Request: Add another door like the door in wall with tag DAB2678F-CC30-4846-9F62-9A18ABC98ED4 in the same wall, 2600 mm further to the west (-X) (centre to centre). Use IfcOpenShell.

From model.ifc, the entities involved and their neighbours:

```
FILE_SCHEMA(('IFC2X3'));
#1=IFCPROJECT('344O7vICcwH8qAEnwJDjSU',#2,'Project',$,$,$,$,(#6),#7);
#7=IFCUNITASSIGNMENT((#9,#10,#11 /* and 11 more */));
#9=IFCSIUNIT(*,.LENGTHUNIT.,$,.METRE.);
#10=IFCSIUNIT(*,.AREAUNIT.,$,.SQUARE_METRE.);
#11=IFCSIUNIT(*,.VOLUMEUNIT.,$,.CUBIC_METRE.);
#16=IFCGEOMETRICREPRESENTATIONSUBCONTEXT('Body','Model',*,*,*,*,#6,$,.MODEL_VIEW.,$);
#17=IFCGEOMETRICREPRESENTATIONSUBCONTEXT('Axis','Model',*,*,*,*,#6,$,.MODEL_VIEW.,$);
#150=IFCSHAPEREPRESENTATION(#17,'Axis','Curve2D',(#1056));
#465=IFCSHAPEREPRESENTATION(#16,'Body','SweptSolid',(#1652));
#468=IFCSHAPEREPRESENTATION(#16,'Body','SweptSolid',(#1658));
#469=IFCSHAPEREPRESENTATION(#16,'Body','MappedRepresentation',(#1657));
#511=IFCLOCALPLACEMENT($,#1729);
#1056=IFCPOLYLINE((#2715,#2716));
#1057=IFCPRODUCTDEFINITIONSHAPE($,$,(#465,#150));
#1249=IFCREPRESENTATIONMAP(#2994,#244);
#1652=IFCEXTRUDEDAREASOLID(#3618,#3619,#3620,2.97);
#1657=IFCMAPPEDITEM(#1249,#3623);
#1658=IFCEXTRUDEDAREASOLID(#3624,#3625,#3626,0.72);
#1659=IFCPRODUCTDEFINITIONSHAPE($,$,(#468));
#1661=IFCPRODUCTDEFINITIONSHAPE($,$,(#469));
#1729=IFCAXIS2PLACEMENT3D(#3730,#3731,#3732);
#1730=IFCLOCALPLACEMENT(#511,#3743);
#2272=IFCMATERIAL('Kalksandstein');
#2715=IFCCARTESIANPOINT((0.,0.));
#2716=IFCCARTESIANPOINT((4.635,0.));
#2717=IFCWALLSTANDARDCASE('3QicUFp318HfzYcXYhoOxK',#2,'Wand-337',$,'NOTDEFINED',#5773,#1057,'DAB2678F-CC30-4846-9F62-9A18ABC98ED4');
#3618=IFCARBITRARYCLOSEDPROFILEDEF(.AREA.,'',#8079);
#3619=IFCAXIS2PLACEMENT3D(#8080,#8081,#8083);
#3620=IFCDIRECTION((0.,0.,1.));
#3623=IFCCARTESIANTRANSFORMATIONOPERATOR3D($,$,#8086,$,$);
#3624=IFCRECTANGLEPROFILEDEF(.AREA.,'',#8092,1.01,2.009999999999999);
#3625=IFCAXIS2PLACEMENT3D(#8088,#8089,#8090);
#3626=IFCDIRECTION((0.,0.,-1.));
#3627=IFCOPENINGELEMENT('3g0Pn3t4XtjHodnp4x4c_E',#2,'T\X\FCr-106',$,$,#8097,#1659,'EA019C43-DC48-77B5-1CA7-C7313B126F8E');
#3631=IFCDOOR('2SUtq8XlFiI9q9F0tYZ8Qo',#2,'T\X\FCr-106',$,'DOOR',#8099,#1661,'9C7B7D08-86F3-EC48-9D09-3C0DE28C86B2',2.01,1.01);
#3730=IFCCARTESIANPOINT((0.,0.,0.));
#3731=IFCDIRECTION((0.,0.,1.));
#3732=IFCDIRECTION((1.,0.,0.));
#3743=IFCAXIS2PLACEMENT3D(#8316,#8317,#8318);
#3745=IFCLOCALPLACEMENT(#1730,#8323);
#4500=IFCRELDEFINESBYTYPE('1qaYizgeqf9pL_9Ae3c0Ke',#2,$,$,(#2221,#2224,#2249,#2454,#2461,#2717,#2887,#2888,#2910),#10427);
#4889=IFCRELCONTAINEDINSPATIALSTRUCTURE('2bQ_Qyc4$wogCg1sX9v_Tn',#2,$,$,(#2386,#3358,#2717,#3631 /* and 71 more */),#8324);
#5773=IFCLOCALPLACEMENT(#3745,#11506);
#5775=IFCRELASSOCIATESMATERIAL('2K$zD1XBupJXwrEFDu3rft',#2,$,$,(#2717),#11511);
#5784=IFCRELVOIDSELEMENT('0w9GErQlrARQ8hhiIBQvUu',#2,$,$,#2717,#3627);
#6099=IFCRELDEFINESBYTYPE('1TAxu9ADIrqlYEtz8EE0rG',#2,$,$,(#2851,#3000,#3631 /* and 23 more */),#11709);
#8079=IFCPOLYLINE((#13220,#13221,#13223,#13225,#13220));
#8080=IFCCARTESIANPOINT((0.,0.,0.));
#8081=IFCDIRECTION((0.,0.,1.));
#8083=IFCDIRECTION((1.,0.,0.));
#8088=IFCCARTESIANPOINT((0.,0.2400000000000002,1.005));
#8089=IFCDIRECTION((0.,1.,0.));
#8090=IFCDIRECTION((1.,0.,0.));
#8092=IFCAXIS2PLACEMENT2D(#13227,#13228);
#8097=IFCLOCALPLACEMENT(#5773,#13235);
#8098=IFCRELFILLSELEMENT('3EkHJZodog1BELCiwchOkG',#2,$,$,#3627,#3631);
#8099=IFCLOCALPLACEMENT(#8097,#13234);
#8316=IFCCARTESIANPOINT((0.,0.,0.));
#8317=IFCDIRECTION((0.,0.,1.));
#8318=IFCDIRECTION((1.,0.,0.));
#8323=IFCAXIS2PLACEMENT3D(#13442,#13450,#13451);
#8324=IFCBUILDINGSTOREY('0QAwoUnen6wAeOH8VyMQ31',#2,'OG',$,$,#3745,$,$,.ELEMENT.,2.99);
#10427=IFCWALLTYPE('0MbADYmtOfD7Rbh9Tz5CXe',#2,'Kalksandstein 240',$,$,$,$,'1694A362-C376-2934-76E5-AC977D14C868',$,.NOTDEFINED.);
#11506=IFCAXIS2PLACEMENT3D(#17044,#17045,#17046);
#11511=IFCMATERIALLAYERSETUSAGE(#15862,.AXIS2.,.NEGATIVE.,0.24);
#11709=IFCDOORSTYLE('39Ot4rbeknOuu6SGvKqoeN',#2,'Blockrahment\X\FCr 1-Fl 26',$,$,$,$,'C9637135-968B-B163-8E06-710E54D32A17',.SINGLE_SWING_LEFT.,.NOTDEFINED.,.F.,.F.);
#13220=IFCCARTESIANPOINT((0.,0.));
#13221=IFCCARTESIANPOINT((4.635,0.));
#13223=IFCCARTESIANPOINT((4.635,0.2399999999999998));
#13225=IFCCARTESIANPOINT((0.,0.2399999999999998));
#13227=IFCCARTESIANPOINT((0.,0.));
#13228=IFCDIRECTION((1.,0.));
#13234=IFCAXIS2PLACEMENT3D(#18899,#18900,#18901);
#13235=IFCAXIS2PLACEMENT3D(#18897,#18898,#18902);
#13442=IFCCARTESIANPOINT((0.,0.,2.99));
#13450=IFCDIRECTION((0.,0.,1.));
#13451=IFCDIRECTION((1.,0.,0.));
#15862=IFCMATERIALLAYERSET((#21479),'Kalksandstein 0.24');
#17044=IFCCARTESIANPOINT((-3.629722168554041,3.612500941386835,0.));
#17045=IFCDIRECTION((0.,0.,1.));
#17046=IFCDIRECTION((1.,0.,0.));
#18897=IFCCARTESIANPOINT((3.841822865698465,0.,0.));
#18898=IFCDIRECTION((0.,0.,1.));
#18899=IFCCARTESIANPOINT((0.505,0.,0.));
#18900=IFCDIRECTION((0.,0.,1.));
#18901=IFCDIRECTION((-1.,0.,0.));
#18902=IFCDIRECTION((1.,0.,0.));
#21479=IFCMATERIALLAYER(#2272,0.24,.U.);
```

```python
import ifcopenshell
import ifcopenshell.api.feature
import ifcopenshell.api.geometry
import ifcopenshell.api.root
import ifcopenshell.geom
import ifcopenshell.util.element
import ifcopenshell.util.placement
import ifcopenshell.util.shape
import ifcopenshell.util.unit

model = ifcopenshell.open("model.ifc")
unit_scale = ifcopenshell.util.unit.calculate_unit_scale(model)
settings = ifcopenshell.geom.settings()


def volume(element):
    """Net volume in cubic metres, openings subtracted."""
    shape = ifcopenshell.geom.create_shape(settings, element)
    return ifcopenshell.util.shape.get_volume(shape.geometry)


def reuse_history(source, copy):
    """copy_class also copies each property set's owner history, people and application; keep the originals."""
    for rel in copy.IsDefinedBy:
        if rel.is_a("IfcRelDefinesByProperties") and (history := rel.RelatingPropertyDefinition.OwnerHistory):
            rel.RelatingPropertyDefinition.OwnerHistory = source.OwnerHistory
            ifcopenshell.util.element.remove_deep2(model, history)


door = model.by_guid("2SUtq8XlFiI9q9F0tYZ8Qo")
opening = door.FillsVoids[0].RelatingOpeningElement
wall = opening.VoidsElements[0].RelatingBuildingElement
before = volume(wall)
shift = ifcopenshell.util.placement.get_local_placement(wall.ObjectPlacement)[:3, 0] * -2.6 / unit_scale

# copy_class copies the void relationship, type, container and properties, but no geometry.
new_opening = ifcopenshell.api.root.copy_class(model, product=opening)
new_opening.Representation = ifcopenshell.util.element.copy_deep(
    model, opening.Representation, exclude=["IfcGeometricRepresentationContext", "IfcRepresentationMap"]
)
new_opening.Tag = None
new_door = ifcopenshell.api.root.copy_class(model, product=door)
new_door.Representation = ifcopenshell.util.element.copy_deep(
    model, door.Representation, exclude=["IfcGeometricRepresentationContext", "IfcRepresentationMap"]
)
new_door.Tag = None
reuse_history(door, new_door)
fills = ifcopenshell.api.feature.add_filling(model, opening=new_opening, element=new_door)
fills.OwnerHistory = new_door.OwnerHistory  # required in IFC2X3

for old, new in ((opening, new_opening), (door, new_door)):
    matrix = ifcopenshell.util.placement.get_local_placement(old.ObjectPlacement)
    matrix[:3, 3] += shift
    ifcopenshell.api.geometry.edit_object_placement(model, product=new, matrix=matrix, is_si=False)

after = volume(wall)

print(f"wall volume {before:.3f} -> {after:.3f} m3")

model.write("model_v2.ifc")
```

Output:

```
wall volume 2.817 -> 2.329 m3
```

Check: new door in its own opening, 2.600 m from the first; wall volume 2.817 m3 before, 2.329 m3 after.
